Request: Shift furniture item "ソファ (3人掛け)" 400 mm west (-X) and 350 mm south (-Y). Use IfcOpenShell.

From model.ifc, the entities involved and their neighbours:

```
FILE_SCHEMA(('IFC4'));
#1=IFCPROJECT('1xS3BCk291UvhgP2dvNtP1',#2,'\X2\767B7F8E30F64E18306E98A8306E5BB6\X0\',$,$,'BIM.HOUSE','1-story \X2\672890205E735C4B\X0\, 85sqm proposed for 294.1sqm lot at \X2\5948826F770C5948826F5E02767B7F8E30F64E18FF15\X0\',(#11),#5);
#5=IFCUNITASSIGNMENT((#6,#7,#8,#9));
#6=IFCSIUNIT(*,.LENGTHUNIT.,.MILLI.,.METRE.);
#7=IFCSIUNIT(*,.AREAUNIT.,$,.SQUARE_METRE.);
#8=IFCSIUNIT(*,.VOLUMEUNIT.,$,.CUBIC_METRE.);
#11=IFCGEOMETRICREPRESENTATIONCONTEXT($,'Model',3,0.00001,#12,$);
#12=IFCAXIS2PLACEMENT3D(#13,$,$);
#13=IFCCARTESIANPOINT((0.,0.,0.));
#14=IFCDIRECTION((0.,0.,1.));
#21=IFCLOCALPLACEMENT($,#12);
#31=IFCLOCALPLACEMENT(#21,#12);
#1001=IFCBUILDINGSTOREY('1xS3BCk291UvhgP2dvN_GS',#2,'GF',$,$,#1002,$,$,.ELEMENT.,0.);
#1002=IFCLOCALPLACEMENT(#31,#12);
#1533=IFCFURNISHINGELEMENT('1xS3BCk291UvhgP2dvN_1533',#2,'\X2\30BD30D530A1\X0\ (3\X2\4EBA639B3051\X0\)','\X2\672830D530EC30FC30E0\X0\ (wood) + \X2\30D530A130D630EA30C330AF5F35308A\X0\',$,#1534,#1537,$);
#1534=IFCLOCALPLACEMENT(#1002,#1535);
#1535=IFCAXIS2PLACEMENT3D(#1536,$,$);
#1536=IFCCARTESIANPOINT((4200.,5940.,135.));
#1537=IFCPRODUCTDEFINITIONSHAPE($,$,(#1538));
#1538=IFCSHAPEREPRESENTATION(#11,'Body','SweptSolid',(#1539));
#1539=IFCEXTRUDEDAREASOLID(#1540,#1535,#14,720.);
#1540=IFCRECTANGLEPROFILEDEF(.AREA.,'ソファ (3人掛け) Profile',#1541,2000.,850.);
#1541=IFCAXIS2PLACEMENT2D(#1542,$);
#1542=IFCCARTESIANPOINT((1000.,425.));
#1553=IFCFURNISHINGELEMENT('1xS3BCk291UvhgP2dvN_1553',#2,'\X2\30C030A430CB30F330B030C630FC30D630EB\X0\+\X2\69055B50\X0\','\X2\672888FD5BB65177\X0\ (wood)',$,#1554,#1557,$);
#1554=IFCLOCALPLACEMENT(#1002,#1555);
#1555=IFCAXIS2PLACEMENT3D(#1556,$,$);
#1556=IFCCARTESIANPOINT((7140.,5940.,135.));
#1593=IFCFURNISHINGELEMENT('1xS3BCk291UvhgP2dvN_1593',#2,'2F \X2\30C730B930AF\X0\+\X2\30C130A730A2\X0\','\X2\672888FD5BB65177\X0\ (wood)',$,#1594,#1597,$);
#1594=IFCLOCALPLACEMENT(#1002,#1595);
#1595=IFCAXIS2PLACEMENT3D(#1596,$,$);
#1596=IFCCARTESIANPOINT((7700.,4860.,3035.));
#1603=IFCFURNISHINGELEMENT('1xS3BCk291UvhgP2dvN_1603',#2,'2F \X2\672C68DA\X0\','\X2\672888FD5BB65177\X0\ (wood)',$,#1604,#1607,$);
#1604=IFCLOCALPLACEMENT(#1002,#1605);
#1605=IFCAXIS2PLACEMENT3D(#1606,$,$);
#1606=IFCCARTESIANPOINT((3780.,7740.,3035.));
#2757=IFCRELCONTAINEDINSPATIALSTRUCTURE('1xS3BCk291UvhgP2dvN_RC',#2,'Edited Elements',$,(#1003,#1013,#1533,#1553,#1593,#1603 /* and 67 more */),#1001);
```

```python
import ifcopenshell
import ifcopenshell.api.geometry
import ifcopenshell.util.placement
import ifcopenshell.util.unit

model = ifcopenshell.open("model.ifc")
unit_scale = ifcopenshell.util.unit.calculate_unit_scale(model)

item = model.by_guid("1xS3BCk291UvhgP2dvN_1533")
matrix = ifcopenshell.util.placement.get_local_placement(item.ObjectPlacement)
matrix[0, 3] -= 0.4 / unit_scale
matrix[1, 3] -= 0.35 / unit_scale
ifcopenshell.api.geometry.edit_object_placement(model, product=item, matrix=matrix, is_si=False)

print(ifcopenshell.util.placement.get_local_placement(item.ObjectPlacement).round(3) + 0.0)

model.write("model_rev.ifc")
```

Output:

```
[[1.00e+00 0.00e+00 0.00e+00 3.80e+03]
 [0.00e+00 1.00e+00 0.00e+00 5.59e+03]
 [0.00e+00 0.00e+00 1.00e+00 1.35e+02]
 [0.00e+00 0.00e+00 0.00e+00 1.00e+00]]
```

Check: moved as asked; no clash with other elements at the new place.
